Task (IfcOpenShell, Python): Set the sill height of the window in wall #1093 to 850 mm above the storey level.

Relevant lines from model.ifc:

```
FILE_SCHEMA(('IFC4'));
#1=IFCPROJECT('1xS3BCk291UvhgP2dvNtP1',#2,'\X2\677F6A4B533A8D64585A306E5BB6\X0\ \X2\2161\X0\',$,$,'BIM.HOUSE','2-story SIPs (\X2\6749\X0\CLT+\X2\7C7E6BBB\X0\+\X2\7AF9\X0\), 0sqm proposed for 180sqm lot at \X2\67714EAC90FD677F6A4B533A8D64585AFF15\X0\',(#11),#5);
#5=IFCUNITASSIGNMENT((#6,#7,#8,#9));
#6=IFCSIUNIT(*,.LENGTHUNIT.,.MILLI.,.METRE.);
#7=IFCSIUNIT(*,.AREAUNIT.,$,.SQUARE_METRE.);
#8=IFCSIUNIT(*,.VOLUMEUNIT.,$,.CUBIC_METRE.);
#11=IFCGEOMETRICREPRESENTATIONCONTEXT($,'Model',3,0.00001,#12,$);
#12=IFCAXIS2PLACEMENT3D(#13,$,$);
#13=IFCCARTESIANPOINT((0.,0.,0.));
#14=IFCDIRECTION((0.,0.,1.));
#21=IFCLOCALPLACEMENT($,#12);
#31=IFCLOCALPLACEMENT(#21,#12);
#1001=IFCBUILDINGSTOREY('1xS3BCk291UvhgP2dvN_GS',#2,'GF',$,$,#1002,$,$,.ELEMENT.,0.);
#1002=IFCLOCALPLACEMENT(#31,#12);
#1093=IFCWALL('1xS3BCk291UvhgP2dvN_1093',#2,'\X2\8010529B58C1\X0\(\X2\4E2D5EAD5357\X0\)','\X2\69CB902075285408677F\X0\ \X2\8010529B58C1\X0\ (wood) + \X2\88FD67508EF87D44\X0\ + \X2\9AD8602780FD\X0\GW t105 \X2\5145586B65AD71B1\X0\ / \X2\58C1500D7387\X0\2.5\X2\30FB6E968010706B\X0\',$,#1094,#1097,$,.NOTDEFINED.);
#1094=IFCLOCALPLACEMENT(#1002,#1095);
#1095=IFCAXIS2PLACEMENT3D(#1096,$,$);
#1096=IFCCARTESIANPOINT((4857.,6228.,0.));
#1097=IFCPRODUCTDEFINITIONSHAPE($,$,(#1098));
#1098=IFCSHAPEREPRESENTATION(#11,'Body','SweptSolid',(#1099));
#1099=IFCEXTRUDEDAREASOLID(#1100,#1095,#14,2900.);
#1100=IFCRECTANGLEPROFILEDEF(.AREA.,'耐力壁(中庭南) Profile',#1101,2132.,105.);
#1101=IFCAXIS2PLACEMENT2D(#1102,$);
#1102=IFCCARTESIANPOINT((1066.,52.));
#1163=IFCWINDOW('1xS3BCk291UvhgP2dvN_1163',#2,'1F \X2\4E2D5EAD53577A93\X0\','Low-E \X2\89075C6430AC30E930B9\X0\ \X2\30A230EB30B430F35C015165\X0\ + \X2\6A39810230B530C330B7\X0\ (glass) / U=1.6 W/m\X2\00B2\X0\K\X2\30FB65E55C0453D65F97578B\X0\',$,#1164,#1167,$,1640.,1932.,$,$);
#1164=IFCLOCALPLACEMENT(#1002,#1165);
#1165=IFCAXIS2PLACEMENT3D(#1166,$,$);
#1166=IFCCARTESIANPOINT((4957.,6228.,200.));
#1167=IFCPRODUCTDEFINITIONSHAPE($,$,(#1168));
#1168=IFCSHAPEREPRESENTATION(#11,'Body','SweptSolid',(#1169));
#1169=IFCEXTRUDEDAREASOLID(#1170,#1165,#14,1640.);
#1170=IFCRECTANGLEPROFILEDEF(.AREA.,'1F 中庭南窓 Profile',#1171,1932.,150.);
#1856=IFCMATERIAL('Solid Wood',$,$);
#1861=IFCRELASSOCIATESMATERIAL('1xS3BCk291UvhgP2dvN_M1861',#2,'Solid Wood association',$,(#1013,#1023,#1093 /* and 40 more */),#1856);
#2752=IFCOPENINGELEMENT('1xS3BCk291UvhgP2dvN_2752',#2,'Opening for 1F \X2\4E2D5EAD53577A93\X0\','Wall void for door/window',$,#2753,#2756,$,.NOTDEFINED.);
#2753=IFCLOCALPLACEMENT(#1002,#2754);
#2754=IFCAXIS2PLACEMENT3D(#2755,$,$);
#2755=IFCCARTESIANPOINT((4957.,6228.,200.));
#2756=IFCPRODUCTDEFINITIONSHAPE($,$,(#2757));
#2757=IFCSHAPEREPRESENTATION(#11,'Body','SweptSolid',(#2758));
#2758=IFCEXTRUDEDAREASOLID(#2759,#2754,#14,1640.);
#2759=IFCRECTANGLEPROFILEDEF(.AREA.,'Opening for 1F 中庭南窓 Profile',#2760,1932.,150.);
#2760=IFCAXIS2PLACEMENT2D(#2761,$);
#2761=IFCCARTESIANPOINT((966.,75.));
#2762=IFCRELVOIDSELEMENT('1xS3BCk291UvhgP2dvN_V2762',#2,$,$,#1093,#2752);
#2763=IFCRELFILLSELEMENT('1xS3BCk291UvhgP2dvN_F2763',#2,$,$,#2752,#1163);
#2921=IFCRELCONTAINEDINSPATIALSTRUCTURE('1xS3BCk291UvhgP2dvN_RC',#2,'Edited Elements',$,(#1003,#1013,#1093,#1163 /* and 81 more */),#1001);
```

```python
import numpy as np
import ifcopenshell
import ifcopenshell.api.geometry
import ifcopenshell.geom
import ifcopenshell.util.element
import ifcopenshell.util.placement
import ifcopenshell.util.shape
import ifcopenshell.util.unit

model = ifcopenshell.open("model.ifc")
unit_scale = ifcopenshell.util.unit.calculate_unit_scale(model)

window = model.by_guid("1xS3BCk291UvhgP2dvN_1163")
opening = window.FillsVoids[0].RelatingOpeningElement
storey = ifcopenshell.util.element.get_container(window, ifc_class="IfcBuildingStorey")
level = ifcopenshell.util.placement.get_local_placement(storey.ObjectPlacement)[2, 3]

# The opening's origin need not be at the sill, so measure its lowest point.
shape = ifcopenshell.geom.create_shape(ifcopenshell.geom.settings(), opening)
bottom = ifcopenshell.util.shape.get_shape_bottom_elevation(shape, shape.geometry) / unit_scale
dz = level + 850.0 - bottom

shift = np.array([0.0, 0.0, dz])
# The window is not placed relative to its opening, so move both.
for product in (opening, window):
    matrix = ifcopenshell.util.placement.get_local_placement(product.ObjectPlacement)
    matrix[:3, 3] += shift
    ifcopenshell.api.geometry.edit_object_placement(model, product=product, matrix=matrix, is_si=False)

print(f"moved by {dz * unit_scale:+.3f} m")

model.write("model_edited.ifc")
```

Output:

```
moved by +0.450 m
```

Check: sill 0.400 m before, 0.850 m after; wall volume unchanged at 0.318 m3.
